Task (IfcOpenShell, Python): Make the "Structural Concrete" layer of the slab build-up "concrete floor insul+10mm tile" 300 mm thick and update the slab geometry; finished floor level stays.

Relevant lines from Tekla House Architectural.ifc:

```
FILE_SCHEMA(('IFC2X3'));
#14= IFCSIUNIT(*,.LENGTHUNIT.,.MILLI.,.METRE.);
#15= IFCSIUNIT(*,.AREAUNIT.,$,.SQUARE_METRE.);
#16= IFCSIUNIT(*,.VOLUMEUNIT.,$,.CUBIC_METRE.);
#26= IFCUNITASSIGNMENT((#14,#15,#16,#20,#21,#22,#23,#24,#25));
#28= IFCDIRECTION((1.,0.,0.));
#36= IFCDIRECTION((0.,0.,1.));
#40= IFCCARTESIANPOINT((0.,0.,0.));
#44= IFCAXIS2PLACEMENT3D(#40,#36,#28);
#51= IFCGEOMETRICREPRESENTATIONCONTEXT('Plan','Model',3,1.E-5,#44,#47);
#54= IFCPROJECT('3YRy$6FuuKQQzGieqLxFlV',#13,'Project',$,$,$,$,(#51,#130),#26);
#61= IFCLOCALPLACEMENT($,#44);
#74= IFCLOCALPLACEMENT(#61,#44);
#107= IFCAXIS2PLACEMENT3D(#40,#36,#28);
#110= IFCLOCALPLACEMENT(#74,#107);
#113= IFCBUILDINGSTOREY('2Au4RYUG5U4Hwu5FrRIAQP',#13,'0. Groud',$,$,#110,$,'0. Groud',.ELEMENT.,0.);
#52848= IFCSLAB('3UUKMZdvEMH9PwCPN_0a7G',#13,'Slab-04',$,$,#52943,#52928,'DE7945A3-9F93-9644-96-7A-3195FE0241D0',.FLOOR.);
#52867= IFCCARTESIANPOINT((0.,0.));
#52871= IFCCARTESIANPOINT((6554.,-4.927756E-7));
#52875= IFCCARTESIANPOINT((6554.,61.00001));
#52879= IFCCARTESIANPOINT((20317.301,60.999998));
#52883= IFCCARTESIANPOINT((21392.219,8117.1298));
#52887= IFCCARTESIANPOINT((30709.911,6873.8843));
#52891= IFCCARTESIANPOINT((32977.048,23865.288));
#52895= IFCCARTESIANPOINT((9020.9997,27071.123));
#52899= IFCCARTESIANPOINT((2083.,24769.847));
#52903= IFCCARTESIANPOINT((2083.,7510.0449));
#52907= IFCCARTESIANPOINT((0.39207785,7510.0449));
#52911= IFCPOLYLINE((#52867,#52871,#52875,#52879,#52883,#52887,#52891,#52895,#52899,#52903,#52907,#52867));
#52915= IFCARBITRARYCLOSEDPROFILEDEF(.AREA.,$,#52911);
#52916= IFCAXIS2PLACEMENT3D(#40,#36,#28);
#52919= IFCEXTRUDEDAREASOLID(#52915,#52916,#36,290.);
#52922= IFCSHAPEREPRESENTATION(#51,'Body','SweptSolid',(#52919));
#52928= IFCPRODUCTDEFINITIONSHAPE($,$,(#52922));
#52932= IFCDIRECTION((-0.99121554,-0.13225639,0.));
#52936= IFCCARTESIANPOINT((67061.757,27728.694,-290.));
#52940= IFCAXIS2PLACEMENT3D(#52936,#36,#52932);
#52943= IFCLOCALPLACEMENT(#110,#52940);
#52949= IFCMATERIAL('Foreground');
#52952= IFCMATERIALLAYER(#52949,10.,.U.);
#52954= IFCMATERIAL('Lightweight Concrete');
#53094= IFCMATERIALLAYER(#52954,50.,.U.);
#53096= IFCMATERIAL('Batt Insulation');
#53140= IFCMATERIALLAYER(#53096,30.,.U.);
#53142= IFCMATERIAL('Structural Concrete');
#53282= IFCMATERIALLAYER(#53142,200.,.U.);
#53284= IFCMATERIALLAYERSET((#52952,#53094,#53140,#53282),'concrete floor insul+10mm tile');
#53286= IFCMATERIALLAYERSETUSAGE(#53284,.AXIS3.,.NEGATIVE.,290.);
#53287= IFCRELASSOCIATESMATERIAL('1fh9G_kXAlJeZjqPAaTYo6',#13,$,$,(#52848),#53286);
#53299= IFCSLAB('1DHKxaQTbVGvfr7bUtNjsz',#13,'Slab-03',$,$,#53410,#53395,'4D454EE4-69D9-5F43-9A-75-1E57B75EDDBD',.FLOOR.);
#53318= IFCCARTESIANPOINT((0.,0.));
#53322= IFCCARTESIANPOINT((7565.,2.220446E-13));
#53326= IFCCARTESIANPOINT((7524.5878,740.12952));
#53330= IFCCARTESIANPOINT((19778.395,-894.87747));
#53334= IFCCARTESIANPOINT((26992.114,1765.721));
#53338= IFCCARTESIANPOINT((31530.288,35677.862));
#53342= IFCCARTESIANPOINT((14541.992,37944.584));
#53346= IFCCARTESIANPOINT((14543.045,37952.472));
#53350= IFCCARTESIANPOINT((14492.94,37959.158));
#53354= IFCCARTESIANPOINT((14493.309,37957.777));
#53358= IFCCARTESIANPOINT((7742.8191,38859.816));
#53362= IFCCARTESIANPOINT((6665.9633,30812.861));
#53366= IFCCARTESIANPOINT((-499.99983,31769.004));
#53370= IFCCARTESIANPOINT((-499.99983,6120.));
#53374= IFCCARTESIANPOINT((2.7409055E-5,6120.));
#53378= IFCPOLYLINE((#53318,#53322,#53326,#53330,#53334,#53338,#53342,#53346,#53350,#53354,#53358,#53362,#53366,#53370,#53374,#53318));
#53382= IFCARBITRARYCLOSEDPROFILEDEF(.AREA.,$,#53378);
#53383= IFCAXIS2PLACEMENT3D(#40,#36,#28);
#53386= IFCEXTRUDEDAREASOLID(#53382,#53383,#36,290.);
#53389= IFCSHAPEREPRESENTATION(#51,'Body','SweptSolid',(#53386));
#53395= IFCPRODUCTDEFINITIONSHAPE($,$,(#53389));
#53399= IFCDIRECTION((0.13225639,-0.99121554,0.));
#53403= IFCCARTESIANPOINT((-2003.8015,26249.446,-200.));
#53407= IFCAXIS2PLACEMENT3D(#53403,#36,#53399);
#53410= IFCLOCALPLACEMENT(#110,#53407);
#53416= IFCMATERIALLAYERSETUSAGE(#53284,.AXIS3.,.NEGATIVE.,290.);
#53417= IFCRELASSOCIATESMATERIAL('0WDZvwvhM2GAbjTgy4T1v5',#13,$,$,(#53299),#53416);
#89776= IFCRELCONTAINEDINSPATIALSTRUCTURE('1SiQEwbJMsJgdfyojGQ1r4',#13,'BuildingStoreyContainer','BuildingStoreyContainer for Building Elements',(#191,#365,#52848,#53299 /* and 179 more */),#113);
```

```python
import ifcopenshell
import ifcopenshell.util.element
import ifcopenshell.util.unit

model = ifcopenshell.open("Tekla House Architectural.ifc")
unit_scale = ifcopenshell.util.unit.calculate_unit_scale(model)

layer_set = model.by_id(53284)
layer = next(l for l in layer_set.MaterialLayers if l.Material and l.Material.Name == "Structural Concrete")
change = 0.3 / unit_scale - layer.LayerThickness
layer.LayerThickness += change

# The layer set is shared, so every slab that uses it gets the new thickness.
slabs = [e for e in ifcopenshell.util.element.get_elements_by_material(model, layer_set) if e.is_a("IfcSlab")]
for slab in sorted(slabs, key=lambda e: e.id()):
    body = next(r for r in slab.Representation.Representations if r.RepresentationIdentifier == "Body")
    solid = body.Items[0]
    old_depth = solid.Depth
    solid.Depth += change
    # Extruded upwards: lower the start of the extrusion so the top stays.
    x, y, z = solid.Position.Location.Coordinates
    solid.Position.Location = model.createIfcCartesianPoint((x, y, z - change))
    print(slab.id(), f"{old_depth:g} -> {solid.Depth:g}")

model.write("Tekla House Architectural_v2.ifc")
```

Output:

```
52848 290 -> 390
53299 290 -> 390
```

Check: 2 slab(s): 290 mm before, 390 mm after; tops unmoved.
